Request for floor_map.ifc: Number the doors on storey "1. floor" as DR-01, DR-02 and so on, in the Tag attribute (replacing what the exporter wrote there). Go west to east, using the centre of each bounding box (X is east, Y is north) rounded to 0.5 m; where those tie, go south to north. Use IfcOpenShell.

First a look at what the model holds.

```python
import ifcopenshell
import ifcopenshell.util.element
import ifcopenshell.util.placement

model = ifcopenshell.open("floor_map.ifc")
print(model.schema)
storey = next(s for s in model.by_type("IfcBuildingStorey") if s.Name == "1. floor")
doors = [e for e in ifcopenshell.util.element.get_decomposition(storey) if e.is_a("IfcDoor")]
for e in sorted(doors, key=lambda e: e.id()):
    origin = ifcopenshell.util.placement.get_local_placement(e.ObjectPlacement)[:3, 3]
    print(e.id(), e.Tag, e.Name, origin.round(2) + 0.0, sep=" | ")
```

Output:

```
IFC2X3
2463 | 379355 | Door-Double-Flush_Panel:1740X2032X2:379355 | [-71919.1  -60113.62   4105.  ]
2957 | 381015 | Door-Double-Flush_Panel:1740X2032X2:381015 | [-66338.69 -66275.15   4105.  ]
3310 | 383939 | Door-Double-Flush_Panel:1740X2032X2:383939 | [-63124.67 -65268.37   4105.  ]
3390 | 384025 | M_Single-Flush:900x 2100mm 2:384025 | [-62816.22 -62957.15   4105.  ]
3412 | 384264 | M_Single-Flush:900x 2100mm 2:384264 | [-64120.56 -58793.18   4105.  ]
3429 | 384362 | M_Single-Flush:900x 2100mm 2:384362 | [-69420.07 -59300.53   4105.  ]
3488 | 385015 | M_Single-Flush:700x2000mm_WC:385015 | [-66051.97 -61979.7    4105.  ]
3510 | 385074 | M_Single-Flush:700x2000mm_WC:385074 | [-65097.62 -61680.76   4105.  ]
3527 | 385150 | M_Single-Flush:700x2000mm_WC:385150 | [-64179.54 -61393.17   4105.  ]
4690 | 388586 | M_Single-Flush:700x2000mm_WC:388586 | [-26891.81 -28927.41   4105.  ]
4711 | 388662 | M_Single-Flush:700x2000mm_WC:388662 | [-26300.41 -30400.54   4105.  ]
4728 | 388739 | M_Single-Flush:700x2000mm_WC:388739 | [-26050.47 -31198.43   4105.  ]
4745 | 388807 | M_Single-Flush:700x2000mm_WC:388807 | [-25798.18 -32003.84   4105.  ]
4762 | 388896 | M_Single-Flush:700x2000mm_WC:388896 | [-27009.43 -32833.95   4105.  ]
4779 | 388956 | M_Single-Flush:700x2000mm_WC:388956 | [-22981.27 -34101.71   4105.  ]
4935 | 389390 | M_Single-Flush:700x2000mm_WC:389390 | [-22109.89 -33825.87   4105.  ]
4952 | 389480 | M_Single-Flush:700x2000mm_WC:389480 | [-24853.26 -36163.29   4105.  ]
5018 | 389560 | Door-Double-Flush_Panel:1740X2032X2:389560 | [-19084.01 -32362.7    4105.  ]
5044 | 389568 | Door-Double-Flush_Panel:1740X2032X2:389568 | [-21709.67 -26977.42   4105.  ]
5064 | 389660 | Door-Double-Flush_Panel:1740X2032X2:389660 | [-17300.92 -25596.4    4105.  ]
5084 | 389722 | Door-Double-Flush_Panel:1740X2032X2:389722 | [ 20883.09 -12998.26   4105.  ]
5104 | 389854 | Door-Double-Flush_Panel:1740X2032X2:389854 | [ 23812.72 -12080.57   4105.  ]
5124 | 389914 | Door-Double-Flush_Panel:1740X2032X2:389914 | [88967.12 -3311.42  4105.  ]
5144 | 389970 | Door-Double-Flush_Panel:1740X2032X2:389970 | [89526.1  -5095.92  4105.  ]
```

```python
import ifcopenshell
import ifcopenshell.geom
import ifcopenshell.util.element
import ifcopenshell.util.shape

model = ifcopenshell.open("floor_map.ifc")
settings = ifcopenshell.geom.settings()
settings.set("use-world-coords", True)


def centre(element):
    shape = ifcopenshell.geom.create_shape(settings, element)
    return ifcopenshell.util.shape.get_bbox_centroid(shape.geometry)


storey = next(s for s in model.by_type("IfcBuildingStorey") if s.Name == "1. floor")
doors = [e for e in ifcopenshell.util.element.get_decomposition(storey) if e.is_a("IfcDoor")]

# Insertion points can sit at a corner or the storey origin, so sort by the geometry (in metres).
centres = {e: centre(e) for e in doors}
doors.sort(key=lambda e: (round(centres[e][0] / 0.5), centres[e][1]))

for i, e in enumerate(doors, start=1):
    number = f"DR-{i:02d}"
    e.Tag = number
    print(e.id(), number)

model.write("floor_map_edited.ifc")
```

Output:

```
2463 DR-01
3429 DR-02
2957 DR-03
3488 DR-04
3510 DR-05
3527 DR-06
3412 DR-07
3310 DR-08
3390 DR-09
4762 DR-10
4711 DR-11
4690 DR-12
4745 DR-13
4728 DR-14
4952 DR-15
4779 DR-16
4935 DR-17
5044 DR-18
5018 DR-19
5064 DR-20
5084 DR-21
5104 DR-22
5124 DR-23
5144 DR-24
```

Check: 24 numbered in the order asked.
